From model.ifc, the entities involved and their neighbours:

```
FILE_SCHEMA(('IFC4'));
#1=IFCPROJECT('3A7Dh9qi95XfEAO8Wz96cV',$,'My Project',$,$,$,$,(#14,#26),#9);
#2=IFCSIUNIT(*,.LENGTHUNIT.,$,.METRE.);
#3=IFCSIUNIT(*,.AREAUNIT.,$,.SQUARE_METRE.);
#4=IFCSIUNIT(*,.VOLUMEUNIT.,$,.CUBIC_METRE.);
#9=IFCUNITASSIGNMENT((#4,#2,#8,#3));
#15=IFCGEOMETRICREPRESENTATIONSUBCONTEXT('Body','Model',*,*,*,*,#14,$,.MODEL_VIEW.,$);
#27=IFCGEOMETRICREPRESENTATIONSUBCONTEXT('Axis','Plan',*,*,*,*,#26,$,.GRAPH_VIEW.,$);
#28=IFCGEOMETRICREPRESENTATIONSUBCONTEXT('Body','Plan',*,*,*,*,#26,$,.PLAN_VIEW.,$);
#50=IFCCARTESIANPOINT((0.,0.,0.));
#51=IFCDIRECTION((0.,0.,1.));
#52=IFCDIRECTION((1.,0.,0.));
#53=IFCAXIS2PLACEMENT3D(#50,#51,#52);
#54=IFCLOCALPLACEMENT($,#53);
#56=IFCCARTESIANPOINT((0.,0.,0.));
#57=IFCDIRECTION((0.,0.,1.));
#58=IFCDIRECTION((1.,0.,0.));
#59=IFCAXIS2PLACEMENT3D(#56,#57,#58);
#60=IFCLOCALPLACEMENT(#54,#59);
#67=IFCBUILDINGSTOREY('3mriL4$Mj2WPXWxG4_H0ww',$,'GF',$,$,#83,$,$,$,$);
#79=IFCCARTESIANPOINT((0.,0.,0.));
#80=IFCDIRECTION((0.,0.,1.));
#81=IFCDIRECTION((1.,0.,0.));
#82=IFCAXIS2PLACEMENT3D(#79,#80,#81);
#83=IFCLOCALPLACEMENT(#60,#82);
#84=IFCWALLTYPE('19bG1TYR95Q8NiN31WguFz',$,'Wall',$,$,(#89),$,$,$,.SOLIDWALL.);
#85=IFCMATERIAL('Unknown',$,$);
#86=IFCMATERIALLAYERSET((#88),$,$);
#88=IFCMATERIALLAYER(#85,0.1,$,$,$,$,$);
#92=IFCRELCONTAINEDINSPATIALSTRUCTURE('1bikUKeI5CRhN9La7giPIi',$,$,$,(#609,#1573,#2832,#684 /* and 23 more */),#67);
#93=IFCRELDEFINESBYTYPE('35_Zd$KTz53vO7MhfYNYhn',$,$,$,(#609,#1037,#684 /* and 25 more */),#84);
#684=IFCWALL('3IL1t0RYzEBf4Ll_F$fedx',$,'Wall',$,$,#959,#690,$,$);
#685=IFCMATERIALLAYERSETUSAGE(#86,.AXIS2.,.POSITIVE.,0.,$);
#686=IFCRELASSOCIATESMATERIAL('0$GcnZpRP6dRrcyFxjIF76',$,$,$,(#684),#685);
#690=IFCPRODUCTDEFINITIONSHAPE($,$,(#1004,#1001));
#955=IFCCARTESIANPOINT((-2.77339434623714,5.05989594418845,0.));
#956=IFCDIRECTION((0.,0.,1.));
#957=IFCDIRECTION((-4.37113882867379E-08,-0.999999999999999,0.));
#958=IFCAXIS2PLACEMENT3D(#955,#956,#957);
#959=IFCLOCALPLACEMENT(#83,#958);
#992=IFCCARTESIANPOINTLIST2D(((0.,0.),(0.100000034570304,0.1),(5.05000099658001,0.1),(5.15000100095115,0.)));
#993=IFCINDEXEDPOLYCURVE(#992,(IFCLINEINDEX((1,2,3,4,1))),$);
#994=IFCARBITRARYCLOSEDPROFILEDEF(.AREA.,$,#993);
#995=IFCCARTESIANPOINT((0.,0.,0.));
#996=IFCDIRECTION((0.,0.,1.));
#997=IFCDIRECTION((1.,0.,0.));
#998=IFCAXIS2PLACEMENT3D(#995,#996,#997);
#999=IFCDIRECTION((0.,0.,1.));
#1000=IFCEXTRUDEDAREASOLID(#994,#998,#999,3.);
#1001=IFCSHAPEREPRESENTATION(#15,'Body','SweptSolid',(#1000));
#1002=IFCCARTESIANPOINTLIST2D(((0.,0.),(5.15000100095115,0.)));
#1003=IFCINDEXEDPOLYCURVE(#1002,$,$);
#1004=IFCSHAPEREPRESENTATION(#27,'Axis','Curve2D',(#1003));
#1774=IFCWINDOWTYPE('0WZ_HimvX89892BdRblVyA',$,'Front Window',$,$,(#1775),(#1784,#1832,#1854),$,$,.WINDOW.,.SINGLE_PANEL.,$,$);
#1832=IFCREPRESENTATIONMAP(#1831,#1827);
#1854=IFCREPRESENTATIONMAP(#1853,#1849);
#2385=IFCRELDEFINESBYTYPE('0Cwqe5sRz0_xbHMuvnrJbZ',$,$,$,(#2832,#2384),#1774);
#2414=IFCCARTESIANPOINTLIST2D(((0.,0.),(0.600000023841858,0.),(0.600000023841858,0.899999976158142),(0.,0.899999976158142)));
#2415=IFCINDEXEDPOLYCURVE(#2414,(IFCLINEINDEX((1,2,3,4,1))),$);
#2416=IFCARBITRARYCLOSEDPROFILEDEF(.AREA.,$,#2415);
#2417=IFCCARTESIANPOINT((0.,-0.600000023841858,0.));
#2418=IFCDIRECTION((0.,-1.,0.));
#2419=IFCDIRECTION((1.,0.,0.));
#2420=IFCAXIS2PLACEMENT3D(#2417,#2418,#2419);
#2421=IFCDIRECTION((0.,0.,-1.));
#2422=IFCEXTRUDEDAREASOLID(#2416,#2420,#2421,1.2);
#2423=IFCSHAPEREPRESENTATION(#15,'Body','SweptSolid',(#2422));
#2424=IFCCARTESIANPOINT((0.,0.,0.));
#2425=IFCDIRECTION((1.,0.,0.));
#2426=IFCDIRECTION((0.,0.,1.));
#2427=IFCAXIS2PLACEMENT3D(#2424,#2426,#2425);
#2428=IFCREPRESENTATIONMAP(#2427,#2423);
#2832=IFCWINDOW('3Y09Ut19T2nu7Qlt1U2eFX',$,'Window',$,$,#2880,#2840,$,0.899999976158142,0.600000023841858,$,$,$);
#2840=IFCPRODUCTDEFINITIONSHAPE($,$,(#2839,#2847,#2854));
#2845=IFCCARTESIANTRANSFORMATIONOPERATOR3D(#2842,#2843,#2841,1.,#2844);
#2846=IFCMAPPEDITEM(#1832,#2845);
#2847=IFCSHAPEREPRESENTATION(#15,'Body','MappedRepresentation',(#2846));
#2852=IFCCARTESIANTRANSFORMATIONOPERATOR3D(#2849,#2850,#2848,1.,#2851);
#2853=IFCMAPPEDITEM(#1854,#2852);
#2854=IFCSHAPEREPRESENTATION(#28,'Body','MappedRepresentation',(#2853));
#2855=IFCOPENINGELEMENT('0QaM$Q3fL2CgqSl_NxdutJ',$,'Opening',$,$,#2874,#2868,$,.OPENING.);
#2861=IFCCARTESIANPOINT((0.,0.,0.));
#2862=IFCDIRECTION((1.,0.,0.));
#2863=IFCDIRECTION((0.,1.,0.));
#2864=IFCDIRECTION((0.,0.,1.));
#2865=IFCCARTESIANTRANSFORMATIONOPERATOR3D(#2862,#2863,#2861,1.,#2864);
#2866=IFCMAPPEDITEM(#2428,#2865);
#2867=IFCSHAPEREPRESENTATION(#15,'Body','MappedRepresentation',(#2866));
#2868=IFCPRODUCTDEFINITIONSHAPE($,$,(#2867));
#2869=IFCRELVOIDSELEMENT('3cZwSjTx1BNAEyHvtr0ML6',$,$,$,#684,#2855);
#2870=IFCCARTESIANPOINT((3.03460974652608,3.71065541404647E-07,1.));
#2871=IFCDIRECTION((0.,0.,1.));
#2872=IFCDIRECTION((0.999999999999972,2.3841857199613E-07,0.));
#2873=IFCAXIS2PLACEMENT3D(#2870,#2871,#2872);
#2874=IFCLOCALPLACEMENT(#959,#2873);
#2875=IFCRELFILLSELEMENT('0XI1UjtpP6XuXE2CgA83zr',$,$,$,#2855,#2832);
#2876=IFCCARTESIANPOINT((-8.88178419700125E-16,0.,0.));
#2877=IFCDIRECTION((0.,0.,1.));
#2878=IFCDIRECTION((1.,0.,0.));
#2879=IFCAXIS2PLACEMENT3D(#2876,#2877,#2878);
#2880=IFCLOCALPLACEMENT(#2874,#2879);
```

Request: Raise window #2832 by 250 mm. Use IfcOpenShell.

```python
import numpy as np
import ifcopenshell
import ifcopenshell.api.geometry
import ifcopenshell.util.placement
import ifcopenshell.util.unit

model = ifcopenshell.open("model.ifc")
unit_scale = ifcopenshell.util.unit.calculate_unit_scale(model)

window = model.by_guid("3Y09Ut19T2nu7Qlt1U2eFX")
opening = window.FillsVoids[0].RelatingOpeningElement
dz = 0.25

shift = np.array([0.0, 0.0, dz])
# The window is placed relative to its opening, so it follows when the opening moves.
matrix = ifcopenshell.util.placement.get_local_placement(opening.ObjectPlacement)
matrix[:3, 3] += shift
ifcopenshell.api.geometry.edit_object_placement(
    model, product=opening, matrix=matrix, is_si=False, should_transform_children=True
)

print(f"moved by {dz * unit_scale:+.3f} m")

model.write("model_v2.ifc")
```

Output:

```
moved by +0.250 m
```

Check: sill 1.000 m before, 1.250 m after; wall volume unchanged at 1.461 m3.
